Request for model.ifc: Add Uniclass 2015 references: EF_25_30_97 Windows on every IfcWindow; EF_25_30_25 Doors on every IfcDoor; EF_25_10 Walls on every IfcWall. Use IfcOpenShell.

First a look at what the model holds.

```python
import ifcopenshell

model = ifcopenshell.open("model.ifc")
print(model.schema)
print("classifications:", [c.Name for c in model.by_type("IfcClassification")])
for ifc_class in ("IfcDoor", "IfcRoof", "IfcStair", "IfcWall", "IfcWindow"):
    print(ifc_class, len(model.by_type(ifc_class)))
```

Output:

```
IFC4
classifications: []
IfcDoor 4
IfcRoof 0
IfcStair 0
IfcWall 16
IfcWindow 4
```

```python
import ifcopenshell
import ifcopenshell.api.classification

model = ifcopenshell.open("model.ifc")

system = ifcopenshell.api.classification.add_classification(model, classification="Uniclass 2015")

codes = {
    "IfcWindow": ("EF_25_30_97", "Windows"),
    "IfcDoor": ("EF_25_30_25", "Doors"),
    "IfcWall": ("EF_25_10", "Walls"),
}
for ifc_class, (code, name) in codes.items():
    products = model.by_type(ifc_class)
    ifcopenshell.api.classification.add_reference(
        model, products=products, classification=system, identification=code, name=name
    )
    print(code, len(products))

model.write("model_v2.ifc")
```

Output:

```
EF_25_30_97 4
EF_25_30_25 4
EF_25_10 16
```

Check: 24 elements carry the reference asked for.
